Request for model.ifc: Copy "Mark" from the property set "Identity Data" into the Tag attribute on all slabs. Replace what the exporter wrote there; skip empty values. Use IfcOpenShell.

First a look at what the model holds.

```python
import ifcopenshell
import ifcopenshell.util.element

model = ifcopenshell.open("model.ifc")
print(model.schema)
slabs = model.by_type("IfcSlab")
print(len(slabs), "slabs")
for e in slabs[:8]:
    source = ifcopenshell.util.element.get_pset(e, "Identity Data", "Mark")
    target = e.Tag
    print(e.id(), repr(source), repr(target), sep=" | ")
```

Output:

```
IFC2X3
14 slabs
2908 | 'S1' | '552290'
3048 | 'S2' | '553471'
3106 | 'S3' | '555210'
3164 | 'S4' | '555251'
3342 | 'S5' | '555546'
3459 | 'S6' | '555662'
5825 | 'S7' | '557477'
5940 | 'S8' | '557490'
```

```python
import ifcopenshell
import ifcopenshell.util.element

model = ifcopenshell.open("model.ifc")

count = 0
for e in model.by_type("IfcSlab"):
    value = ifcopenshell.util.element.get_pset(e, "Identity Data", "Mark")
    current = e.Tag
    if not value or not value.strip() or current == value:
        continue
    e.Tag = value
    count += 1

print(count, "slabs updated")

model.write("model-out.ifc")
```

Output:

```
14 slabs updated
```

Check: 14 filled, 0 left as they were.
